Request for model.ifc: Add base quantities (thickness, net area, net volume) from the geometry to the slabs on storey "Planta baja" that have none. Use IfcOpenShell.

First a look at what the model holds.

```python
import ifcopenshell
import ifcopenshell.util.element
import ifcopenshell.util.unit

model = ifcopenshell.open("model.ifc")
print(model.schema)
for unit_type in ("LENGTHUNIT", "AREAUNIT", "VOLUMEUNIT"):
    print(unit_type, ifcopenshell.util.unit.calculate_unit_scale(model, unit_type))
storey = next(s for s in model.by_type("IfcBuildingStorey") if s.Name == "Planta baja")
slabs = [e for e in ifcopenshell.util.element.get_decomposition(storey) if e.is_a("IfcSlab")]
for e in sorted(slabs, key=lambda e: e.id()):
    print(e.id(), e.is_a(), e.Name, list(ifcopenshell.util.element.get_psets(e, qtos_only=True)), sep=" | ")
```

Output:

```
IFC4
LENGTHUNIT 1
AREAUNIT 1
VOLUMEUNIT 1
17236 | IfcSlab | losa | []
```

```python
import ifcopenshell
import ifcopenshell.api.pset
import ifcopenshell.geom
import ifcopenshell.util.element
import ifcopenshell.util.shape
import ifcopenshell.util.unit

model = ifcopenshell.open("model.ifc")
unit_scale = ifcopenshell.util.unit.calculate_unit_scale(model)
area_scale = ifcopenshell.util.unit.calculate_unit_scale(model, "AREAUNIT")
volume_scale = ifcopenshell.util.unit.calculate_unit_scale(model, "VOLUMEUNIT")
settings = ifcopenshell.geom.settings()

storey = next(s for s in model.by_type("IfcBuildingStorey") if s.Name == "Planta baja")
slabs = [e for e in ifcopenshell.util.element.get_decomposition(storey) if e.is_a("IfcSlab")]

for e in sorted(slabs, key=lambda e: e.id()):
    if ifcopenshell.util.element.get_psets(e, qtos_only=True, should_inherit=False):
        continue
    # Geometry comes back in metres, in the element's own axes.
    shape = ifcopenshell.geom.create_shape(settings, e)
    values = {
        "Width": ifcopenshell.util.shape.get_z(shape.geometry) / unit_scale,
        "NetArea": ifcopenshell.util.shape.get_footprint_area(shape.geometry) / area_scale,
        "NetVolume": ifcopenshell.util.shape.get_volume(shape.geometry) / volume_scale,
    }
    qto = ifcopenshell.api.pset.add_qto(model, product=e, name="Qto_SlabBaseQuantities")
    ifcopenshell.api.pset.edit_qto(model, qto=qto, properties=values)
    print(e.id(), {k: round(v, 3) for k, v in values.items()})

model.write("model_rev.ifc")
```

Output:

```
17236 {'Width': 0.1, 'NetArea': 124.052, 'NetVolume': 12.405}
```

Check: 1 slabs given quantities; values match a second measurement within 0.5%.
